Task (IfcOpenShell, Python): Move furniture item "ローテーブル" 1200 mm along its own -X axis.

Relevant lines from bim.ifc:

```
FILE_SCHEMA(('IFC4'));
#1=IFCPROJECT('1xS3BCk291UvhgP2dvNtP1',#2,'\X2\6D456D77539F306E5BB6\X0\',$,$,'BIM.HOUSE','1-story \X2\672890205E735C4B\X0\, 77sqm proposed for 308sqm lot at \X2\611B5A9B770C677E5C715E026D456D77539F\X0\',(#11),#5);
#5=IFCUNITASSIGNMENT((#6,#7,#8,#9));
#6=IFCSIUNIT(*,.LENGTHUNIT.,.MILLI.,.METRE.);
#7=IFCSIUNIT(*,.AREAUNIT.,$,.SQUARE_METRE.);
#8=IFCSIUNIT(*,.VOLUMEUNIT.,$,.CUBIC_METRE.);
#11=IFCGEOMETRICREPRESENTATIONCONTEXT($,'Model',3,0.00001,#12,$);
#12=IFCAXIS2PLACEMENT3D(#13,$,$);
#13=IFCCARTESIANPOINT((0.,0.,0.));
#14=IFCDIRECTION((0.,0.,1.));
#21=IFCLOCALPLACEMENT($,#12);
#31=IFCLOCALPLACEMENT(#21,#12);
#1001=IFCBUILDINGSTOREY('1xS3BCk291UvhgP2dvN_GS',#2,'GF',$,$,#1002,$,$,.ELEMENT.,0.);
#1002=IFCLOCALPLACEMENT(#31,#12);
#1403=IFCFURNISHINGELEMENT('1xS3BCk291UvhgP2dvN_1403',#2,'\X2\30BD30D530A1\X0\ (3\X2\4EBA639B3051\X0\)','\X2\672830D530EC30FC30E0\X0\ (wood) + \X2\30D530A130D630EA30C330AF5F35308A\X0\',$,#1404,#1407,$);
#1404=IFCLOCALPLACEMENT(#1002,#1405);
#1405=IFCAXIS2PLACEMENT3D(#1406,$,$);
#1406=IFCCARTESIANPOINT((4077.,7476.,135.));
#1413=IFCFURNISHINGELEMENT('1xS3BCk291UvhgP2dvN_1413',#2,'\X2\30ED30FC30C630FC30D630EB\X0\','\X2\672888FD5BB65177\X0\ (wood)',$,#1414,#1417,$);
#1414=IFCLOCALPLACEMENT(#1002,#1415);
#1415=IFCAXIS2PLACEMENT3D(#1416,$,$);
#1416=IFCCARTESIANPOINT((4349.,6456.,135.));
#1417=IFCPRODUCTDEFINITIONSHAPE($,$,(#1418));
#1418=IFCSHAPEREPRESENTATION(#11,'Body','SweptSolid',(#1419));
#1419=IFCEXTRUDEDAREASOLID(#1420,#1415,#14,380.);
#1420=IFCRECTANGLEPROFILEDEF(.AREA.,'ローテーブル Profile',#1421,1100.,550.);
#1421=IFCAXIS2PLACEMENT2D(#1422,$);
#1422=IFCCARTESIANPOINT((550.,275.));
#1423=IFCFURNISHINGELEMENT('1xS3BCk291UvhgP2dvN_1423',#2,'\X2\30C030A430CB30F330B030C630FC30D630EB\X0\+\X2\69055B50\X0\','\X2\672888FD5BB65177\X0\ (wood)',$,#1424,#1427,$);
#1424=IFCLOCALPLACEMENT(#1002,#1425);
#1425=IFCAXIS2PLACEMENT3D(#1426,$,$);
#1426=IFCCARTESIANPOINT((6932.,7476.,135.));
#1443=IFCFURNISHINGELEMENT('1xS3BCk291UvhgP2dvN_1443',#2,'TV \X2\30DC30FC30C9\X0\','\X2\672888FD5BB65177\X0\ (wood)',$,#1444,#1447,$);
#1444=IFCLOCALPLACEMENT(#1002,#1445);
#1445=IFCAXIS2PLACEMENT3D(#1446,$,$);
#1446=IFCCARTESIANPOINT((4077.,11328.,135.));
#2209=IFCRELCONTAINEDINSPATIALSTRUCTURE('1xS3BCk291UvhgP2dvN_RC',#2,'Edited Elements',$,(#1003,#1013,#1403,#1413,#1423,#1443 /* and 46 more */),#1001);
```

```python
import ifcopenshell
import ifcopenshell.api.geometry
import ifcopenshell.util.placement

model = ifcopenshell.open("bim.ifc")

item = model.by_guid("1xS3BCk291UvhgP2dvN_1413")
matrix = ifcopenshell.util.placement.get_local_placement(item.ObjectPlacement)
matrix[:3, 3] -= matrix[:3, 0] * 1200.0
ifcopenshell.api.geometry.edit_object_placement(model, product=item, matrix=matrix, is_si=False)

print(ifcopenshell.util.placement.get_local_placement(item.ObjectPlacement).round(3) + 0.0)

model.write("bim_v2.ifc")
```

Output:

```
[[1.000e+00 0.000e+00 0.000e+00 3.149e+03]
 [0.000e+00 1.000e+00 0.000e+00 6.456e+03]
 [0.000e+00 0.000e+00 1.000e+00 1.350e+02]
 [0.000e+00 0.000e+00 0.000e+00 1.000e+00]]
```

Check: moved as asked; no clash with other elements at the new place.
